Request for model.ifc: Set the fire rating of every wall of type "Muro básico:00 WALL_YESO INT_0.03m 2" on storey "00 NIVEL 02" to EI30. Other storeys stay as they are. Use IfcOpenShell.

First a look at what the model holds.

```python
import ifcopenshell
import ifcopenshell.util.element

model = ifcopenshell.open("model.ifc")
print(model.schema)
storey = next(s for s in model.by_type("IfcBuildingStorey") if s.Name == "00 NIVEL 02")
walls = [e for e in ifcopenshell.util.element.get_decomposition(storey) if e.is_a("IfcWall")]
seen = {}
for e in walls:
    element_type = ifcopenshell.util.element.get_type(e)
    key = (element_type.Name if element_type != e and element_type else None, ifcopenshell.util.element.get_pset(e, "Pset_WallCommon", "FireRating"))
    seen[key] = seen.get(key, 0) + 1
for (name, value), count in sorted(seen.items(), key=str):
    print(count, "x", name, "|", value)
```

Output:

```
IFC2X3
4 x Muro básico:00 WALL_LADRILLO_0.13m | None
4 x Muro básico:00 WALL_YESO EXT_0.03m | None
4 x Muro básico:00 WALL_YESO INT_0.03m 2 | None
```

```python
import ifcopenshell
import ifcopenshell.api.pset
import ifcopenshell.util.element

model = ifcopenshell.open("model.ifc")

storey = next(s for s in model.by_type("IfcBuildingStorey") if s.Name == "00 NIVEL 02")
walls = [e for e in ifcopenshell.util.element.get_decomposition(storey) if e.is_a("IfcWall")]

count = 0
for e in walls:
    element_type = ifcopenshell.util.element.get_type(e)
    if element_type in (None, e) or element_type.Name != "Muro básico:00 WALL_YESO INT_0.03m 2":
        continue
    # add_pset returns the element's existing set when there is one.
    pset = ifcopenshell.api.pset.add_pset(model, product=e, name="Pset_WallCommon")
    ifcopenshell.api.pset.edit_pset(model, pset=pset, properties={"FireRating": "EI30"})
    count += 1

print(count, "walls updated")

model.write("model_v2.ifc")
```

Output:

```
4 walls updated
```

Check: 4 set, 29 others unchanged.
